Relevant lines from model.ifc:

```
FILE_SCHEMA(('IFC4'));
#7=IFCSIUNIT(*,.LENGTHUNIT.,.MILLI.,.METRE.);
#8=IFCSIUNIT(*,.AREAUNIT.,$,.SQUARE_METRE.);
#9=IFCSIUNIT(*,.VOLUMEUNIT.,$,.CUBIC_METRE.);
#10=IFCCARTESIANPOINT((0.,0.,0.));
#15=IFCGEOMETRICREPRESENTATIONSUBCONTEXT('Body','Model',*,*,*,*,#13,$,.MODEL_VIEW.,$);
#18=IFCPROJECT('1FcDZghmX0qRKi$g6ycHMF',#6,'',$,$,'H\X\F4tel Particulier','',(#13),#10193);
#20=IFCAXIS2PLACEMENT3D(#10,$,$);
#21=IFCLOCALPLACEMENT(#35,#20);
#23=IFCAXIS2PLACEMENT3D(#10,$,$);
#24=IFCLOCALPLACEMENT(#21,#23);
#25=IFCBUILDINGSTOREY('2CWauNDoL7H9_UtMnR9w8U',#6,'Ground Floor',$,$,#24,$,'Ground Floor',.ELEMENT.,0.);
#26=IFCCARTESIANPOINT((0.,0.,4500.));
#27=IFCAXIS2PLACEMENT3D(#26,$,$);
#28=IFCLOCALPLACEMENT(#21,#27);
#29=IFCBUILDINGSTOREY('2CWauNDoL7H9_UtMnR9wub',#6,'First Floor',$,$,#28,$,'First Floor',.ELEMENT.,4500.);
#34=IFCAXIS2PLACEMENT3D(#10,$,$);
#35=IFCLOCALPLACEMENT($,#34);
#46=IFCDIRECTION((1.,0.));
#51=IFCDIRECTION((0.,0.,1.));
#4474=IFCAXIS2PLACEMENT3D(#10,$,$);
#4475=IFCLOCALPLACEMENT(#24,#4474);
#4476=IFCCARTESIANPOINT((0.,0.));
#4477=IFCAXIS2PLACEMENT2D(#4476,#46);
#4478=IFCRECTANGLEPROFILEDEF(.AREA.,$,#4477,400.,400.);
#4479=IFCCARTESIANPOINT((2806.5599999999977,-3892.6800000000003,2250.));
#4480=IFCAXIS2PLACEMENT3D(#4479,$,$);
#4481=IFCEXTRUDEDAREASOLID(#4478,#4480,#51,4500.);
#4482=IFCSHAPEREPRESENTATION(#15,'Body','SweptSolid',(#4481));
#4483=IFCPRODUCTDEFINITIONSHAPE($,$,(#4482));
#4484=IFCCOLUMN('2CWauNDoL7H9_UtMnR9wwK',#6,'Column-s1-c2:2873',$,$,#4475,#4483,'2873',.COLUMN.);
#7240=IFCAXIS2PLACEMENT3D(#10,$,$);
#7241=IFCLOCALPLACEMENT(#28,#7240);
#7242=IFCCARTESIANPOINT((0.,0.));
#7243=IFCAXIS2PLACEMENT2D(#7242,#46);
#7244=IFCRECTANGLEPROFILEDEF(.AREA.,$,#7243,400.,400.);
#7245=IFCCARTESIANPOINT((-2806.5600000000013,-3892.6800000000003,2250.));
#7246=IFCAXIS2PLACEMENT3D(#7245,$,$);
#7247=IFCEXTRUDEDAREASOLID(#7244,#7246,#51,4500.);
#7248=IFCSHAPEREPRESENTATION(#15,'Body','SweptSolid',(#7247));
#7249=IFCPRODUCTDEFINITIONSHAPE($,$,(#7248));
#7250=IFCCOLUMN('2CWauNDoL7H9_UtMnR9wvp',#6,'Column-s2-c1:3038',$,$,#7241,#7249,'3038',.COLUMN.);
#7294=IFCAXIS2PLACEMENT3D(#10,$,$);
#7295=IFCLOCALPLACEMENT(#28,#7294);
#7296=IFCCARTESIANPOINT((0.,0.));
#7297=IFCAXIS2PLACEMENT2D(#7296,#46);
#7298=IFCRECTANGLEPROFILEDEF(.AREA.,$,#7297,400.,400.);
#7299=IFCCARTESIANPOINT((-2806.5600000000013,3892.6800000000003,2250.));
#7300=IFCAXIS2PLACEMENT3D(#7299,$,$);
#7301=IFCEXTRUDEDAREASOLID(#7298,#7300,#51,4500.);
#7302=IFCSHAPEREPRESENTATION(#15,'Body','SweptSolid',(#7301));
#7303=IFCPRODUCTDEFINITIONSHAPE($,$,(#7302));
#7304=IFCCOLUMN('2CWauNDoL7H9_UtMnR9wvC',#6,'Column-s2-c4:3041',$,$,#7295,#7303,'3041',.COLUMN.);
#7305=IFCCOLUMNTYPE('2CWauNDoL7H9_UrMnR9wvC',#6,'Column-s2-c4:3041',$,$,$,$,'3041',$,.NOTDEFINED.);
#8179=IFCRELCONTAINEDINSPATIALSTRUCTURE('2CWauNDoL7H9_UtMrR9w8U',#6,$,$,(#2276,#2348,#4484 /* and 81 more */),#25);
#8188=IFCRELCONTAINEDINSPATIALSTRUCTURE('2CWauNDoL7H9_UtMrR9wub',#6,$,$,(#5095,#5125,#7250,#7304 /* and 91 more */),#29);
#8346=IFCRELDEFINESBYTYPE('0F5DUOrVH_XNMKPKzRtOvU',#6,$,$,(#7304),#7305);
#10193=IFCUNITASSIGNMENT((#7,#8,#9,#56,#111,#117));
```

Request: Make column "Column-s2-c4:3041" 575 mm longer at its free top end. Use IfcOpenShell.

```python
import ifcopenshell
import ifcopenshell.util.representation

model = ifcopenshell.open("model.ifc")

member = model.by_guid("2CWauNDoL7H9_UtMnR9wvC")
change = 575.0

# The extrusion runs towards the end named, so only its depth changes.
body = ifcopenshell.util.representation.get_representation(member, "Model", "Body")
solid = body.Items[0]
old_length = solid.Depth
solid.Depth += change

print(f"length {old_length:g} -> {solid.Depth:g}")

model.write("model_edited.ifc")
```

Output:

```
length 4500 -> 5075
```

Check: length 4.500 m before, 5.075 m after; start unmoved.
